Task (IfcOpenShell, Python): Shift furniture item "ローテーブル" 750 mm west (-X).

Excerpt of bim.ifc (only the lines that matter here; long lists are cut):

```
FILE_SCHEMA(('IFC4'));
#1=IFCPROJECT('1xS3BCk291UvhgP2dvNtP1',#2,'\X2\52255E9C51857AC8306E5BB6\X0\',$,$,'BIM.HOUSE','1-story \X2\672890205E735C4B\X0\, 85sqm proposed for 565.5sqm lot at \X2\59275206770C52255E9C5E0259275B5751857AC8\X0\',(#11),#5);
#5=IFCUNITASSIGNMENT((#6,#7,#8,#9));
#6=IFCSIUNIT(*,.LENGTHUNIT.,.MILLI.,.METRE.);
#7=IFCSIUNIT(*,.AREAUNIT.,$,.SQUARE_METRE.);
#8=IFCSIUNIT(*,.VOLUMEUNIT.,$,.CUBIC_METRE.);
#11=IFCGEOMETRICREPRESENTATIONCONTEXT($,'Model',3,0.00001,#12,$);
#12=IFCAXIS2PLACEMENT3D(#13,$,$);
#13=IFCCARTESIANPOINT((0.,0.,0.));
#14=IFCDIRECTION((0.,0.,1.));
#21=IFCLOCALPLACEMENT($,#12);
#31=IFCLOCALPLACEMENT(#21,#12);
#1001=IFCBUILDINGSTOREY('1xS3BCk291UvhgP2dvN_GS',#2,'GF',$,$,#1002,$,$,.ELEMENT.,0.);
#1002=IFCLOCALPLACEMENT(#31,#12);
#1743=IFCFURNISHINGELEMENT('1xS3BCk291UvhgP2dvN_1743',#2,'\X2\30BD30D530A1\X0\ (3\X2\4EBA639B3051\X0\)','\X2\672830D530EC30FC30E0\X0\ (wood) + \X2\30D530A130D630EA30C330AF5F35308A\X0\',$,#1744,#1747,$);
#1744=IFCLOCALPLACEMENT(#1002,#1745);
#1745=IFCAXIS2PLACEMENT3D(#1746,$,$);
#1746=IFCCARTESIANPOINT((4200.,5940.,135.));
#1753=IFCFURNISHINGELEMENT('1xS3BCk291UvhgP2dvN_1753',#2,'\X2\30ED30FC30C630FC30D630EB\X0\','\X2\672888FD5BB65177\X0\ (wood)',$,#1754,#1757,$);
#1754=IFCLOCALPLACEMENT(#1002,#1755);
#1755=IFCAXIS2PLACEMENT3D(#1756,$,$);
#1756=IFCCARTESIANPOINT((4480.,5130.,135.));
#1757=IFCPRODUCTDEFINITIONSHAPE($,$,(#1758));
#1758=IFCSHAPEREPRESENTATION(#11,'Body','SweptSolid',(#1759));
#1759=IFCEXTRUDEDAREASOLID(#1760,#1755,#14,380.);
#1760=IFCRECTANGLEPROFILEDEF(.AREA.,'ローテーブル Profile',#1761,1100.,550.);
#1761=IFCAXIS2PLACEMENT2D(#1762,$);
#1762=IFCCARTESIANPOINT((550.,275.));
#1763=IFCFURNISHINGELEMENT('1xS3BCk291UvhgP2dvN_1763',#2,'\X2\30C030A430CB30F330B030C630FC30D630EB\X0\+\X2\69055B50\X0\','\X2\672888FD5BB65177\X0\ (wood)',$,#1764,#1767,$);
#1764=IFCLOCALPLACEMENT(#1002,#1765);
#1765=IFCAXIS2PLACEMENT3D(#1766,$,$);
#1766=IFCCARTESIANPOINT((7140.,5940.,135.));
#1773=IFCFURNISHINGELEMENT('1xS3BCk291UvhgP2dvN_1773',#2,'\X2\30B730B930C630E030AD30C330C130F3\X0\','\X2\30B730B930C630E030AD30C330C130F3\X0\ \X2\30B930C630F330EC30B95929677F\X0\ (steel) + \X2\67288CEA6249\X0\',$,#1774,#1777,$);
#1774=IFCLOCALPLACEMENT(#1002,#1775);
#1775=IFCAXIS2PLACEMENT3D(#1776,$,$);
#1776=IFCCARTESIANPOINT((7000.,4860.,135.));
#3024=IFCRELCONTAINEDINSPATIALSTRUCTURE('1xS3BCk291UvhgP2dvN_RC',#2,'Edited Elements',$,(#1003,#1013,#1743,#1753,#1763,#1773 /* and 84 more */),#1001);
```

```python
import ifcopenshell
import ifcopenshell.api.geometry
import ifcopenshell.util.placement

model = ifcopenshell.open("bim.ifc")

item = model.by_guid("1xS3BCk291UvhgP2dvN_1753")
matrix = ifcopenshell.util.placement.get_local_placement(item.ObjectPlacement)
matrix[0, 3] -= 750.0
ifcopenshell.api.geometry.edit_object_placement(model, product=item, matrix=matrix, is_si=False)

print(ifcopenshell.util.placement.get_local_placement(item.ObjectPlacement).round(3) + 0.0)

model.write("bim-out.ifc")
```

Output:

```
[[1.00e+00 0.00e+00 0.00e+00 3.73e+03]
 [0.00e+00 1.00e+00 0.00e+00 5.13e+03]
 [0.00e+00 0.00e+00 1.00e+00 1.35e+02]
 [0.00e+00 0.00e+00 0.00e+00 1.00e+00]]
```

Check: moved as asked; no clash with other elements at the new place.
